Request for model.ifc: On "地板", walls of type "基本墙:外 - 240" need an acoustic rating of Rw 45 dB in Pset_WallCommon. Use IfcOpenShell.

First a look at what the model holds.

```python
import ifcopenshell
import ifcopenshell.util.element

model = ifcopenshell.open("model.ifc")
print(model.schema)
storey = next(s for s in model.by_type("IfcBuildingStorey") if s.Name == "地板")
walls = [e for e in ifcopenshell.util.element.get_decomposition(storey) if e.is_a("IfcWall")]
seen = {}
for e in walls:
    element_type = ifcopenshell.util.element.get_type(e)
    key = (element_type.Name if element_type != e and element_type else None, ifcopenshell.util.element.get_pset(e, "Pset_WallCommon", "AcousticRating"))
    seen[key] = seen.get(key, 0) + 1
for (name, value), count in sorted(seen.items(), key=str):
    print(count, "x", name, "|", value)
```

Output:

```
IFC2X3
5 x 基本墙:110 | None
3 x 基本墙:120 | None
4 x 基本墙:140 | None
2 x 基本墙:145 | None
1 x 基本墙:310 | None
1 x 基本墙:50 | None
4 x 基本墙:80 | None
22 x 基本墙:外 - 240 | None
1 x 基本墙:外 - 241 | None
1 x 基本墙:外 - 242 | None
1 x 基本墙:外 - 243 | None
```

```python
import ifcopenshell
import ifcopenshell.api.pset
import ifcopenshell.util.element

model = ifcopenshell.open("model.ifc")

storey = next(s for s in model.by_type("IfcBuildingStorey") if s.Name == "地板")
walls = [e for e in ifcopenshell.util.element.get_decomposition(storey) if e.is_a("IfcWall")]

count = 0
for e in walls:
    element_type = ifcopenshell.util.element.get_type(e)
    if element_type in (None, e) or element_type.Name != "基本墙:外 - 240":
        continue
    # add_pset returns the element's existing set when there is one.
    pset = ifcopenshell.api.pset.add_pset(model, product=e, name="Pset_WallCommon")
    ifcopenshell.api.pset.edit_pset(model, pset=pset, properties={"AcousticRating": "Rw 45 dB"})
    count += 1

print(count, "walls updated")

model.write("model_edited.ifc")
```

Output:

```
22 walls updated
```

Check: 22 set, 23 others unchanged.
